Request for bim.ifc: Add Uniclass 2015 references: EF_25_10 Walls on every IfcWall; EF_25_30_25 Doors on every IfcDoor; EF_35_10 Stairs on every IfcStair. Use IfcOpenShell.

First a look at what the model holds.

```python
import ifcopenshell

model = ifcopenshell.open("bim.ifc")
print(model.schema)
print("classifications:", [c.Name for c in model.by_type("IfcClassification")])
for ifc_class in ("IfcDoor", "IfcRoof", "IfcStair", "IfcWall", "IfcWindow"):
    print(ifc_class, len(model.by_type(ifc_class)))
```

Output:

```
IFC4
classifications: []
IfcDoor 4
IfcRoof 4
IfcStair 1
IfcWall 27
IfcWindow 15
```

```python
import ifcopenshell
import ifcopenshell.api.classification

model = ifcopenshell.open("bim.ifc")

system = ifcopenshell.api.classification.add_classification(model, classification="Uniclass 2015")

codes = {
    "IfcWall": ("EF_25_10", "Walls"),
    "IfcDoor": ("EF_25_30_25", "Doors"),
    "IfcStair": ("EF_35_10", "Stairs"),
}
for ifc_class, (code, name) in codes.items():
    products = model.by_type(ifc_class)
    ifcopenshell.api.classification.add_reference(
        model, products=products, classification=system, identification=code, name=name
    )
    print(code, len(products))

model.write("bim-out.ifc")
```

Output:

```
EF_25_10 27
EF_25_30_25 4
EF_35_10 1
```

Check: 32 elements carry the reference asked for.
